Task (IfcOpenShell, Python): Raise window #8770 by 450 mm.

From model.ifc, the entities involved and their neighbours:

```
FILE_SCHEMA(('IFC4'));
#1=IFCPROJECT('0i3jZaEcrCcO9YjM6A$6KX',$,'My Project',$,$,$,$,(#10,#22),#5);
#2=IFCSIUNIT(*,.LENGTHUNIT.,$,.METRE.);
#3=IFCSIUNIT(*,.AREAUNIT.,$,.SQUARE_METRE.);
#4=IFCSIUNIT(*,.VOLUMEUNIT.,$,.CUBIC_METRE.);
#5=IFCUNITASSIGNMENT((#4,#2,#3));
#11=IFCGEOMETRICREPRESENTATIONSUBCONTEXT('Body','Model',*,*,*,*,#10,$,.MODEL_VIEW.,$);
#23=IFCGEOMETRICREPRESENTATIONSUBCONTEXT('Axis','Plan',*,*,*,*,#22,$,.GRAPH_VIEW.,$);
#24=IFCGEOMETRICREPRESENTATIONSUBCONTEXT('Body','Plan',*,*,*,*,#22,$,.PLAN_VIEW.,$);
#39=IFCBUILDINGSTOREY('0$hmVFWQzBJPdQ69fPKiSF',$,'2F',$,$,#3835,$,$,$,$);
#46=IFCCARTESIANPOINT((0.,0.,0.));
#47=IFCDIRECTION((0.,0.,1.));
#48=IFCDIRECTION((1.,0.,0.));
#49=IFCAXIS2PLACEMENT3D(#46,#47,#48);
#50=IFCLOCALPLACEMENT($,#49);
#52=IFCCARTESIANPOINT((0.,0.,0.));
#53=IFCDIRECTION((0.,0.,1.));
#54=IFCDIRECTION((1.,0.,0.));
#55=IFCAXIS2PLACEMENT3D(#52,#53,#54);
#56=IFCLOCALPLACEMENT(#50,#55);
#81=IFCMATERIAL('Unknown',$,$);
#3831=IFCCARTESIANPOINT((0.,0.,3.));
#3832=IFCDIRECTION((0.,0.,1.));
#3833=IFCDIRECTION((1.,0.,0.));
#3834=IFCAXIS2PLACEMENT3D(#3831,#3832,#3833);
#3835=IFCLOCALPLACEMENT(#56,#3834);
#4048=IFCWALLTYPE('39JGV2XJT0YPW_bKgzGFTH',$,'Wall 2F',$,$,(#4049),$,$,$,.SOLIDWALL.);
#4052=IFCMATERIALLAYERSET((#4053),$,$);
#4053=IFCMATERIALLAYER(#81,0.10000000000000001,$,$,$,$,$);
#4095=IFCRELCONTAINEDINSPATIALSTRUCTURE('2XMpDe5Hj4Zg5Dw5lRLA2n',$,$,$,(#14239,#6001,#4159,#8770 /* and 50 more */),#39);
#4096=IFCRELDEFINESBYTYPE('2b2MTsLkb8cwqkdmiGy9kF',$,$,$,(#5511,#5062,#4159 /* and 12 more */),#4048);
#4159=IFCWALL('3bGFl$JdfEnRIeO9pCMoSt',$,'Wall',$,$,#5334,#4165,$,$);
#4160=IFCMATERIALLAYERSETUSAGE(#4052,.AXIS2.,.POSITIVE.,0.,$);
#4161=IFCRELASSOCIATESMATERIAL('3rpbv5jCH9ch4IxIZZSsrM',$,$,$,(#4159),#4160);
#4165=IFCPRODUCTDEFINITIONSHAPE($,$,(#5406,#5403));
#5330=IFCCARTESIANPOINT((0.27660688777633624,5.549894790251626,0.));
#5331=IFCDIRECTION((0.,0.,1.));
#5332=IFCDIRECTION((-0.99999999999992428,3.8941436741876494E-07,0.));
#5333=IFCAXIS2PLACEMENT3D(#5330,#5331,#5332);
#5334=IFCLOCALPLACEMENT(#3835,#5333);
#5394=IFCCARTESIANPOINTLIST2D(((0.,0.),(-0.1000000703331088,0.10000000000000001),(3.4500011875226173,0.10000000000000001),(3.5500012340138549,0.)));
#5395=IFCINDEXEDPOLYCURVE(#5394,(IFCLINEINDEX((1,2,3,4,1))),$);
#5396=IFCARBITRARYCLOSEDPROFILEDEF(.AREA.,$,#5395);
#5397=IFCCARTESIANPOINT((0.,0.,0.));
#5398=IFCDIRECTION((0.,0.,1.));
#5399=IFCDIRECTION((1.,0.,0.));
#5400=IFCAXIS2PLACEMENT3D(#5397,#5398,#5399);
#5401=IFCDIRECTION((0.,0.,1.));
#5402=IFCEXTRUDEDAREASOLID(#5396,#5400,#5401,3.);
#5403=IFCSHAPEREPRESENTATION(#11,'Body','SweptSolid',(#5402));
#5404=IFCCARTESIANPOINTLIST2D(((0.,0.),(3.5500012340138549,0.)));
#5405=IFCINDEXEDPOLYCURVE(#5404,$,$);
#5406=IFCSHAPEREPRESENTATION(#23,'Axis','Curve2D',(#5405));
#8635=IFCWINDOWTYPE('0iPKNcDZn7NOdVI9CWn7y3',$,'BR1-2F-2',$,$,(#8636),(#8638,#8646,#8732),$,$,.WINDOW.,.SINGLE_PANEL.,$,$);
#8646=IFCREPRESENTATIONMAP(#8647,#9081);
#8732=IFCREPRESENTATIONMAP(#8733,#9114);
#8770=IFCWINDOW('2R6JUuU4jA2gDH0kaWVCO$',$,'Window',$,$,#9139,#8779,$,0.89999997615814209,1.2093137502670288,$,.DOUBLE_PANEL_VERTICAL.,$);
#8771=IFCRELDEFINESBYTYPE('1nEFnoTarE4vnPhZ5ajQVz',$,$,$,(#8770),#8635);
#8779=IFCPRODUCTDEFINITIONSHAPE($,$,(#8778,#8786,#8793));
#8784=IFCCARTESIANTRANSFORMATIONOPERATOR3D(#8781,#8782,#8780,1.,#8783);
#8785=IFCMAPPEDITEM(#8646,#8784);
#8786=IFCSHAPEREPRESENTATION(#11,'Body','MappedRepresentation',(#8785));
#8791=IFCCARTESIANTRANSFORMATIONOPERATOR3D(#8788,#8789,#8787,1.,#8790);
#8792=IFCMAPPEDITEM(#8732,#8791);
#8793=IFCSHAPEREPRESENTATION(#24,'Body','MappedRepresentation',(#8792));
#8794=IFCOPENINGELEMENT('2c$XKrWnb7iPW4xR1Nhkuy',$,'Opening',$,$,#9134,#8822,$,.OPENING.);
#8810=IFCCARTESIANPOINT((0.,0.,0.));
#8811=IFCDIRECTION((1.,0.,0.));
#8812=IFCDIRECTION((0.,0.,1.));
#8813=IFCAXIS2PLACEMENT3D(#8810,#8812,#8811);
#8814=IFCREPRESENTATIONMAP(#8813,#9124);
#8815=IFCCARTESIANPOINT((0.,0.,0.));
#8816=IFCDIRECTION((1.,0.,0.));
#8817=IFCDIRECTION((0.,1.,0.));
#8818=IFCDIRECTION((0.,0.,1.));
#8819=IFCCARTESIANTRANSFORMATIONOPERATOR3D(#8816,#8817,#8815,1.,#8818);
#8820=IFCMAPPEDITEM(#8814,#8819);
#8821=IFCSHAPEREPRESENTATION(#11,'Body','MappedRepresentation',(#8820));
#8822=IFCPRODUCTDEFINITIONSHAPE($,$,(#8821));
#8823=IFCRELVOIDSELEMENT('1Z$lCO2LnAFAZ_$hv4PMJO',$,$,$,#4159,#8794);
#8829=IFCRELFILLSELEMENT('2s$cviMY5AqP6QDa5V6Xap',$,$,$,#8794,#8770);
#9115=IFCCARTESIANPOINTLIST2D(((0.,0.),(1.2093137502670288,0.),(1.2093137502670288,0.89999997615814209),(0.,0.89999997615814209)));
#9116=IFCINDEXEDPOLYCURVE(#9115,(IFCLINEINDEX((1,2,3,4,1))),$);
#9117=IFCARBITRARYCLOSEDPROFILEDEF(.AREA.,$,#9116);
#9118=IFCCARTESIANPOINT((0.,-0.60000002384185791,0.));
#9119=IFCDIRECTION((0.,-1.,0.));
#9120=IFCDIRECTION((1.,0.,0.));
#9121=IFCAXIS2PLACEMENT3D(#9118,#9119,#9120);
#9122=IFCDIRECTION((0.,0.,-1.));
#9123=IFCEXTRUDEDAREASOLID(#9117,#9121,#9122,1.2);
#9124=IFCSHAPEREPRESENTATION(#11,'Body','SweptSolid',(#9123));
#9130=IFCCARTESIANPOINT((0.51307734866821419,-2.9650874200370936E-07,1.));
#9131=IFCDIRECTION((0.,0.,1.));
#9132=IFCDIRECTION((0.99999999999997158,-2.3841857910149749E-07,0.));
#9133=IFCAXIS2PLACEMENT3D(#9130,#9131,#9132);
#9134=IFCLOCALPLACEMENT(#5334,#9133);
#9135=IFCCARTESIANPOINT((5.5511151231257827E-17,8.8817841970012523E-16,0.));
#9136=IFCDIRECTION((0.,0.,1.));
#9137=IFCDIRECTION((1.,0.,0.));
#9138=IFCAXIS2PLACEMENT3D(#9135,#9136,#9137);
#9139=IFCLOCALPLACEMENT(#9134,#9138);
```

```python
import numpy as np
import ifcopenshell
import ifcopenshell.api.geometry
import ifcopenshell.util.placement
import ifcopenshell.util.unit

model = ifcopenshell.open("model.ifc")
unit_scale = ifcopenshell.util.unit.calculate_unit_scale(model)

window = model.by_id(8770)
opening = window.FillsVoids[0].RelatingOpeningElement
dz = 0.45 / unit_scale

shift = np.array([0.0, 0.0, dz])
# The window is placed relative to its opening, so it follows when the opening moves.
matrix = ifcopenshell.util.placement.get_local_placement(opening.ObjectPlacement)
matrix[:3, 3] += shift
ifcopenshell.api.geometry.edit_object_placement(
    model, product=opening, matrix=matrix, is_si=False, should_transform_children=True
)

print(f"moved by {dz * unit_scale:+.3f} m")

model.write("model_rev.ifc")
```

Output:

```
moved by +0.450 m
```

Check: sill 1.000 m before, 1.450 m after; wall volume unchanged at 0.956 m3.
